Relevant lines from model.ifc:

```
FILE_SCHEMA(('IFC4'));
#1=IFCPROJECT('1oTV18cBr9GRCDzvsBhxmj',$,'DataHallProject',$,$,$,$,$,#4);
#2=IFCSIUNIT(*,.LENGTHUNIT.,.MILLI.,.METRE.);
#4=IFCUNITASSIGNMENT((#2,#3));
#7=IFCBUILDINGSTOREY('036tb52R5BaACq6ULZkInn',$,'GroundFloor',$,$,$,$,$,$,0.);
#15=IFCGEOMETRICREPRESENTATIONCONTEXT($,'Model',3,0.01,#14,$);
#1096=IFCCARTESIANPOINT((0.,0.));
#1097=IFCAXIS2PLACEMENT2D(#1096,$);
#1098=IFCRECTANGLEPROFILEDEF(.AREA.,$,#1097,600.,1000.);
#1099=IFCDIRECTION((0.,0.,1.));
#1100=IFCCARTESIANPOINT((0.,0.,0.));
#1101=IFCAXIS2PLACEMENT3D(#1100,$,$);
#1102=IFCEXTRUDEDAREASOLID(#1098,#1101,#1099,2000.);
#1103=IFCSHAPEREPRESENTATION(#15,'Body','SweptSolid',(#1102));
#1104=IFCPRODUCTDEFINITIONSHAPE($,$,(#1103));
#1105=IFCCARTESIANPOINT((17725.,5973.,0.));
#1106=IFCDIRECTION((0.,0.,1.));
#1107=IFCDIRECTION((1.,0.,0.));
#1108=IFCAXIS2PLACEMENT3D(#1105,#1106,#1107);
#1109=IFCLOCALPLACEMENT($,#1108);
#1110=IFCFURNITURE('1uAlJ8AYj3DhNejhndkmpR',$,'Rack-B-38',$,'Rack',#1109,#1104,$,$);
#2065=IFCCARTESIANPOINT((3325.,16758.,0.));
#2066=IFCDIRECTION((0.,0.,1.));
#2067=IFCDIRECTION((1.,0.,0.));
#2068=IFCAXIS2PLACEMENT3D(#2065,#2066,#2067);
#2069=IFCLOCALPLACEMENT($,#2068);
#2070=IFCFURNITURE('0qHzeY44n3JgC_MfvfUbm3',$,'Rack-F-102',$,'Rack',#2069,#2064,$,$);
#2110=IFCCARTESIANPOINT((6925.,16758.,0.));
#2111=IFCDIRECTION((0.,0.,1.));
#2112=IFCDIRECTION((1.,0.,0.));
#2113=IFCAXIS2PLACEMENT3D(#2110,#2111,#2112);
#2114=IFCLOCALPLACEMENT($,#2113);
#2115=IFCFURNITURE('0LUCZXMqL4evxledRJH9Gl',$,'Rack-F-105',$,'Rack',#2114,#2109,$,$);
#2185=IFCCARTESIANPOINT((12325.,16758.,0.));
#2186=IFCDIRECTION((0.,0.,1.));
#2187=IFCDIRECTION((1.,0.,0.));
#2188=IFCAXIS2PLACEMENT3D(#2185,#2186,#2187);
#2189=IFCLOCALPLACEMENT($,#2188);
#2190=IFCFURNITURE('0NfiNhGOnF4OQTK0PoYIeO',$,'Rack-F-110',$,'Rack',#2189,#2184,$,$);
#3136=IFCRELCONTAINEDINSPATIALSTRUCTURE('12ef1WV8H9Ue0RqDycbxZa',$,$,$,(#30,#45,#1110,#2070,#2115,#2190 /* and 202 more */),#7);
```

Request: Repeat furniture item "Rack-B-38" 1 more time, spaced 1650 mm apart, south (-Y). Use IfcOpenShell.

```python
import numpy as np
import ifcopenshell
import ifcopenshell.api.geometry
import ifcopenshell.api.root
import ifcopenshell.util.element
import ifcopenshell.util.placement

model = ifcopenshell.open("model.ifc")

source = model.by_id(1110)
base = ifcopenshell.util.placement.get_local_placement(source.ObjectPlacement)
step = np.array([0.0, -1.0, 0.0]) * 1650.0

for i in range(1, 2):
    copy = ifcopenshell.api.root.copy_class(model, product=source)
    copy.Representation = ifcopenshell.util.element.copy_deep(
        model, source.Representation, exclude=["IfcGeometricRepresentationContext", "IfcRepresentationMap"]
    )
    matrix = base.copy()
    matrix[:3, 3] += i * step
    print("added at", matrix[:3, 3].round(3) + 0.0)
    ifcopenshell.api.geometry.edit_object_placement(model, product=copy, matrix=matrix, is_si=False)

model.write("model-out.ifc")
```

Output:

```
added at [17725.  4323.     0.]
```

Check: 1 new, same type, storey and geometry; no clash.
